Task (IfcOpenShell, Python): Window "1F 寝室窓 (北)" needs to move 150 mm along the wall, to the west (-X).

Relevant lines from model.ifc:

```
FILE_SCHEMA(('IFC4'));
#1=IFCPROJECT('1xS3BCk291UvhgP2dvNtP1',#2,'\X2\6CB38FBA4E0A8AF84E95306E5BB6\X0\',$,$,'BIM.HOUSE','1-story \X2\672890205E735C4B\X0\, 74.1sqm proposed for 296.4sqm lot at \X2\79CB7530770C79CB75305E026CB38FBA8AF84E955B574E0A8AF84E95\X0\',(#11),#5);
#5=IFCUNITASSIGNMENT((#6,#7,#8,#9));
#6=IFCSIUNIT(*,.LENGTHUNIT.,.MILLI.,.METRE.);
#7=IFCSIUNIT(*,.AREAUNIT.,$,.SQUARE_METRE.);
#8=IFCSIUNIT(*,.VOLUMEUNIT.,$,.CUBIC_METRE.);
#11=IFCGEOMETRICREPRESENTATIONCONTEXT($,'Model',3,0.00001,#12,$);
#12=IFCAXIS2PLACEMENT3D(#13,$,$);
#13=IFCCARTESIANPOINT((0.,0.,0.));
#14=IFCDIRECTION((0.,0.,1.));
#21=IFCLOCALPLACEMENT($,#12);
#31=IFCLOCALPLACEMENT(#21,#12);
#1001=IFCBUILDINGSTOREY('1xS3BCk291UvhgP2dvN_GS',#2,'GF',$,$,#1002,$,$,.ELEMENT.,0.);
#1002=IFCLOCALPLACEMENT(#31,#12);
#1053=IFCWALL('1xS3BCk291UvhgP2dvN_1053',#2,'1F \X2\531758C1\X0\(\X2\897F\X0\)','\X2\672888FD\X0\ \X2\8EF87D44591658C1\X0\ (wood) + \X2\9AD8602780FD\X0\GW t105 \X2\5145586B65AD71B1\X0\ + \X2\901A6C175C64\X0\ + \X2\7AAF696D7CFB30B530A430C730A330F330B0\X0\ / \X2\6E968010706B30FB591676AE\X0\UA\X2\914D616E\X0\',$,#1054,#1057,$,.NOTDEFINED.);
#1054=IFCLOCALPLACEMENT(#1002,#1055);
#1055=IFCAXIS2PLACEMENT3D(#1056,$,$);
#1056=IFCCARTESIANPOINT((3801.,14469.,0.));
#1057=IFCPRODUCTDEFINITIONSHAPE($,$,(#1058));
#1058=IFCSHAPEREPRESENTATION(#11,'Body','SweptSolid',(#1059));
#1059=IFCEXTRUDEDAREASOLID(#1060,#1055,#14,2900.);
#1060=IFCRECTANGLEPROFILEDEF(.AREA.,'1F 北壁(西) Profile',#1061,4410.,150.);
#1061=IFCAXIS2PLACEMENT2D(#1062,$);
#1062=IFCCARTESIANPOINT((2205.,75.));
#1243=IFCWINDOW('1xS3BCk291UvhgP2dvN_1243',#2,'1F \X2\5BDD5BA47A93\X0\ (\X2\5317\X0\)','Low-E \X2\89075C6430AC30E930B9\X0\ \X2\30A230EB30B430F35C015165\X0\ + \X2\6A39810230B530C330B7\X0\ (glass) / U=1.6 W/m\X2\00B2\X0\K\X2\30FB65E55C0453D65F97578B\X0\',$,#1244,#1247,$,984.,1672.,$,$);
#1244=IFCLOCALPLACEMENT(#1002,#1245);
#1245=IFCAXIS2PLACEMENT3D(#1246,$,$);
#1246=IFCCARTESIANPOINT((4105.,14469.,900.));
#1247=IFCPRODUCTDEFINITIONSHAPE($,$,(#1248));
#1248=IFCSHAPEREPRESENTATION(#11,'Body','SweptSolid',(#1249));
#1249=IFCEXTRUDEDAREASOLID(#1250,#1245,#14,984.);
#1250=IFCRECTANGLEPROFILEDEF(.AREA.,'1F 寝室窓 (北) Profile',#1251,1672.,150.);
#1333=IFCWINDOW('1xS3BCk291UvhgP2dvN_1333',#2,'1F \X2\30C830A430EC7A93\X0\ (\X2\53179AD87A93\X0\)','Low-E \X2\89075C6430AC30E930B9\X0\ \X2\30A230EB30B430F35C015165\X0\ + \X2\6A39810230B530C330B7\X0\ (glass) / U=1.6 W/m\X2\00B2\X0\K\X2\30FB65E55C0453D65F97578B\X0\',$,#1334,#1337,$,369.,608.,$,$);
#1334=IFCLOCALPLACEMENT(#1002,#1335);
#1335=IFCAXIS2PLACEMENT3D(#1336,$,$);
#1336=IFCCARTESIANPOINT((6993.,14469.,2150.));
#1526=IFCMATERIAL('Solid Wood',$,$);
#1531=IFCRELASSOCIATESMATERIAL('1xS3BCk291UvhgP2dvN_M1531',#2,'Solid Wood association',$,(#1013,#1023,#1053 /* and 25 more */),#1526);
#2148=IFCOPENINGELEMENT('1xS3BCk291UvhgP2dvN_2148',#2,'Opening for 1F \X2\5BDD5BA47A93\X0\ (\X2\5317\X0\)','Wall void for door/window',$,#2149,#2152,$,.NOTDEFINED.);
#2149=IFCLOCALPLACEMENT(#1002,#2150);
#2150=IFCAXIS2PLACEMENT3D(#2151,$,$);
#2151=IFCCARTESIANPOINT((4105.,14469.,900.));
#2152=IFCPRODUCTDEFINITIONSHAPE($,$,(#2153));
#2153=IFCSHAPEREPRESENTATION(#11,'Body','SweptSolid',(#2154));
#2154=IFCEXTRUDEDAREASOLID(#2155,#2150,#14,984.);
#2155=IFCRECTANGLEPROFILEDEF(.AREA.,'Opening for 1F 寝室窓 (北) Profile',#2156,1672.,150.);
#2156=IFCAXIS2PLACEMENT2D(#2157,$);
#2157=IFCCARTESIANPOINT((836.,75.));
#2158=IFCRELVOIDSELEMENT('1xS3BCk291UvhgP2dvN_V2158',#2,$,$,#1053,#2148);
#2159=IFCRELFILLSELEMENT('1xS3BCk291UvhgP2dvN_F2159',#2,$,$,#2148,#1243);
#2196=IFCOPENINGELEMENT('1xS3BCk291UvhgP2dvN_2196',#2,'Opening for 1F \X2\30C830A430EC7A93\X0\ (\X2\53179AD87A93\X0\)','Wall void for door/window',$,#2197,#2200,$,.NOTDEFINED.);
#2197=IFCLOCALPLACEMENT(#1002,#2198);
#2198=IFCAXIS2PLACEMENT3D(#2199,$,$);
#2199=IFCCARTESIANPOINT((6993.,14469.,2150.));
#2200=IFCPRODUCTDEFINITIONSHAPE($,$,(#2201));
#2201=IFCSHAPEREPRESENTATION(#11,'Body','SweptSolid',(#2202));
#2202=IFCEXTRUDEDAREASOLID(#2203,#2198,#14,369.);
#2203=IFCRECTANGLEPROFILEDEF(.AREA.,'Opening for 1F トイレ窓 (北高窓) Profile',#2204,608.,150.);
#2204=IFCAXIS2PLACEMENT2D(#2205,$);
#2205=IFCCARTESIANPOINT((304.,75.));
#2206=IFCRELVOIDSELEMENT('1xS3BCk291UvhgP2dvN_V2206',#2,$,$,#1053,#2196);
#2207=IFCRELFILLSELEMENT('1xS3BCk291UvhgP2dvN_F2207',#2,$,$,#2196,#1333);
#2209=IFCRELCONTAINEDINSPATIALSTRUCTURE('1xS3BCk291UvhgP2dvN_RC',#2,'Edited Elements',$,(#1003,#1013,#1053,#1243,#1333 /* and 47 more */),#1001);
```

```python
import ifcopenshell
import ifcopenshell.api.geometry
import ifcopenshell.util.placement
import ifcopenshell.util.unit

model = ifcopenshell.open("model.ifc")
unit_scale = ifcopenshell.util.unit.calculate_unit_scale(model)

window = model.by_id(1243)
opening = window.FillsVoids[0].RelatingOpeningElement
wall = opening.VoidsElements[0].RelatingBuildingElement

wall_matrix = ifcopenshell.util.placement.get_local_placement(wall.ObjectPlacement)
shift = wall_matrix[:3, 0] * -0.15 / unit_scale
before = ifcopenshell.util.placement.get_local_placement(window.ObjectPlacement)[:3, 3].copy()

# The window is not placed relative to its opening, so move both.
for product in (opening, window):
    matrix = ifcopenshell.util.placement.get_local_placement(product.ObjectPlacement)
    matrix[:3, 3] += shift
    ifcopenshell.api.geometry.edit_object_placement(model, product=product, matrix=matrix, is_si=False)

after = ifcopenshell.util.placement.get_local_placement(window.ObjectPlacement)[:3, 3]
print("window moved by", (after - before).round(3) + 0.0)

model.write("model-out.ifc")
```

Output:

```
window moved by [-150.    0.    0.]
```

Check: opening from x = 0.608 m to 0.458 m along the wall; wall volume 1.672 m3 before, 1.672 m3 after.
